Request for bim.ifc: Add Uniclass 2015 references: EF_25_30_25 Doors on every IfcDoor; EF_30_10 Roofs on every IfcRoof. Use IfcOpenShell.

First a look at what the model holds.

```python
import ifcopenshell

model = ifcopenshell.open("bim.ifc")
print(model.schema)
print("classifications:", [c.Name for c in model.by_type("IfcClassification")])
for ifc_class in ("IfcDoor", "IfcRoof", "IfcStair", "IfcWall", "IfcWindow"):
    print(ifc_class, len(model.by_type(ifc_class)))
```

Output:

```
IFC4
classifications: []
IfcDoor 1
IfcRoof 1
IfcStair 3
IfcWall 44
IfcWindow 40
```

```python
import ifcopenshell
import ifcopenshell.api.classification

model = ifcopenshell.open("bim.ifc")

system = ifcopenshell.api.classification.add_classification(model, classification="Uniclass 2015")

codes = {
    "IfcDoor": ("EF_25_30_25", "Doors"),
    "IfcRoof": ("EF_30_10", "Roofs"),
}
for ifc_class, (code, name) in codes.items():
    products = model.by_type(ifc_class)
    ifcopenshell.api.classification.add_reference(
        model, products=products, classification=system, identification=code, name=name
    )
    print(code, len(products))

model.write("bim_updated.ifc")
```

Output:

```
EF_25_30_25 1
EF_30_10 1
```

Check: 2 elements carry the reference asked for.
